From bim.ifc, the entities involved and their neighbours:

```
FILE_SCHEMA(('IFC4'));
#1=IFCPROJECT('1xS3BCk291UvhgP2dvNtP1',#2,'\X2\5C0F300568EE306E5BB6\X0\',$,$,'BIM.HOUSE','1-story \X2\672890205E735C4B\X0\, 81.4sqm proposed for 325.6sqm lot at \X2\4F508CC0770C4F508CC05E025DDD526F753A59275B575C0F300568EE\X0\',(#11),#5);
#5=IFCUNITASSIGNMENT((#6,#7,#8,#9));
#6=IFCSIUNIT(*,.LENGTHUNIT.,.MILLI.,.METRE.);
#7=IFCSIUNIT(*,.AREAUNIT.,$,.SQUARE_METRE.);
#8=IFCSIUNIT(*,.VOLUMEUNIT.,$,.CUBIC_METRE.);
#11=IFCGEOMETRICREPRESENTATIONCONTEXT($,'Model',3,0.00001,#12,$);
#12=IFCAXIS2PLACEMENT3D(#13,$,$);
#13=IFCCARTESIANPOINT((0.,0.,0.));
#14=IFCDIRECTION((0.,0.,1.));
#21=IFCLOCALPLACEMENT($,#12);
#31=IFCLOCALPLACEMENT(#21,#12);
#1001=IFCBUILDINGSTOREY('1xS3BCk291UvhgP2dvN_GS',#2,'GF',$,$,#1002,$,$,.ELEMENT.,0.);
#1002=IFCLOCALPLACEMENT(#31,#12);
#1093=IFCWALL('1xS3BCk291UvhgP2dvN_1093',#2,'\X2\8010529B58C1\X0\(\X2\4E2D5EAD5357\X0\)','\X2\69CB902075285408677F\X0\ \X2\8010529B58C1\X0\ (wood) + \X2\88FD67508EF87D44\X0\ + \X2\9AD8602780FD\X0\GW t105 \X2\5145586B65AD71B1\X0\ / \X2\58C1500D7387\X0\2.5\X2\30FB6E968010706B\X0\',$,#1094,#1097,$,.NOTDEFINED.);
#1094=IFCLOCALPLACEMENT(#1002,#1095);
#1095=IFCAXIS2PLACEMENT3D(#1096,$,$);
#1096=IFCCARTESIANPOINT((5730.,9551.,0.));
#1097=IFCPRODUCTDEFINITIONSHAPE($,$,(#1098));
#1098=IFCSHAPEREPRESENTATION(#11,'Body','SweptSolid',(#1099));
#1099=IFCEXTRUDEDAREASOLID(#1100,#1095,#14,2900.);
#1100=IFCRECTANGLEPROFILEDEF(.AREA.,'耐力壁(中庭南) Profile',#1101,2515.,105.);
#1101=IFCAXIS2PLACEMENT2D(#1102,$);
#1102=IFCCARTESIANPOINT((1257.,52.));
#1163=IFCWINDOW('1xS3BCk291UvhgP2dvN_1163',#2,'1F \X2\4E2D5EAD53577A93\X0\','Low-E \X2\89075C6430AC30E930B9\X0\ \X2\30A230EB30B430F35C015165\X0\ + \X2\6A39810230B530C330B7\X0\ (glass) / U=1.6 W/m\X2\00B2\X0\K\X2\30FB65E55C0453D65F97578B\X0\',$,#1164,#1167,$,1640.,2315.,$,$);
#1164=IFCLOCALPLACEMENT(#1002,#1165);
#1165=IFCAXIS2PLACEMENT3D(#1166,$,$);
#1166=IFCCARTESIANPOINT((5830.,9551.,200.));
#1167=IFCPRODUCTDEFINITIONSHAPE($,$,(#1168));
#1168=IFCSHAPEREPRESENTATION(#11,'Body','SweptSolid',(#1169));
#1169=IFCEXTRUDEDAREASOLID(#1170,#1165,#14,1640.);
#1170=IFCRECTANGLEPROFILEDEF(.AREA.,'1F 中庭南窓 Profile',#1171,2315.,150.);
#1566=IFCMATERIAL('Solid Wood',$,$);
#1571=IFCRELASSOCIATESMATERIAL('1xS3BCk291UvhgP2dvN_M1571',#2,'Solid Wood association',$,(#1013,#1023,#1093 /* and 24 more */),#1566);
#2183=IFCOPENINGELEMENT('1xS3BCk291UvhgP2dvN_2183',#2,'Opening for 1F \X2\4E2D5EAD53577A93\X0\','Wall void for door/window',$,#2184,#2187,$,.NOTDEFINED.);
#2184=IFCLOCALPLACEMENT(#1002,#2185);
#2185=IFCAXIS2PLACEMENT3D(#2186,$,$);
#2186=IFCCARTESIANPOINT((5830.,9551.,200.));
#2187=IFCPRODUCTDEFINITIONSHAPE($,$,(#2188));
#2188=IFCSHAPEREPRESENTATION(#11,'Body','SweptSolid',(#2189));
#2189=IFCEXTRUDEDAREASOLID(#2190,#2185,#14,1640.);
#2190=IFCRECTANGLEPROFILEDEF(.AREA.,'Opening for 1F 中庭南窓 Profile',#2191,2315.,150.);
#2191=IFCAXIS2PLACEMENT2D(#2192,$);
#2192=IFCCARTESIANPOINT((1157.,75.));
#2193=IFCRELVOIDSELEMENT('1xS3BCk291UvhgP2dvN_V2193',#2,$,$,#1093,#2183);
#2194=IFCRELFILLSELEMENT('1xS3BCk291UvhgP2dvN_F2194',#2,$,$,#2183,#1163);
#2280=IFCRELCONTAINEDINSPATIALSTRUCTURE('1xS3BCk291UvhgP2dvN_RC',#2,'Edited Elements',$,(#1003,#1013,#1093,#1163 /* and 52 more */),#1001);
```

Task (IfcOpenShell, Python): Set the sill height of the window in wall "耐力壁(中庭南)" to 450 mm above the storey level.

```python
import numpy as np
import ifcopenshell
import ifcopenshell.api.geometry
import ifcopenshell.geom
import ifcopenshell.util.element
import ifcopenshell.util.placement
import ifcopenshell.util.shape
import ifcopenshell.util.unit

model = ifcopenshell.open("bim.ifc")
unit_scale = ifcopenshell.util.unit.calculate_unit_scale(model)

window = model.by_id(1163)
opening = window.FillsVoids[0].RelatingOpeningElement
storey = ifcopenshell.util.element.get_container(window, ifc_class="IfcBuildingStorey")
level = ifcopenshell.util.placement.get_local_placement(storey.ObjectPlacement)[2, 3]

# The opening's origin need not be at the sill, so measure its lowest point.
shape = ifcopenshell.geom.create_shape(ifcopenshell.geom.settings(), opening)
bottom = ifcopenshell.util.shape.get_shape_bottom_elevation(shape, shape.geometry) / unit_scale
dz = level + 0.45 / unit_scale - bottom

shift = np.array([0.0, 0.0, dz])
# The window is not placed relative to its opening, so move both.
for product in (opening, window):
    matrix = ifcopenshell.util.placement.get_local_placement(product.ObjectPlacement)
    matrix[:3, 3] += shift
    ifcopenshell.api.geometry.edit_object_placement(model, product=product, matrix=matrix, is_si=False)

print(f"moved by {dz * unit_scale:+.3f} m")

model.write("bim_rev.ifc")
```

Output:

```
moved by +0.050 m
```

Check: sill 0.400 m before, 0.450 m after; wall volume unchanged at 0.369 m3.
